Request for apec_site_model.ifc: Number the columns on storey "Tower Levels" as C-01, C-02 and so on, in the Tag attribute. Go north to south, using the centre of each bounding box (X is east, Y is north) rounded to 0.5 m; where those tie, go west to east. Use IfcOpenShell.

First a look at what the model holds.

```python
import ifcopenshell
import ifcopenshell.util.element
import ifcopenshell.util.placement

model = ifcopenshell.open("apec_site_model.ifc")
print(model.schema)
storey = next(s for s in model.by_type("IfcBuildingStorey") if s.Name == "Tower Levels")
columns = [e for e in ifcopenshell.util.element.get_decomposition(storey) if e.is_a("IfcColumn")]
for e in sorted(columns, key=lambda e: e.id()):
    origin = ifcopenshell.util.placement.get_local_placement(e.ObjectPlacement)[:3, 3]
    print(e.id(), e.Tag, e.Name, origin.round(2) + 0.0, sep=" | ")
```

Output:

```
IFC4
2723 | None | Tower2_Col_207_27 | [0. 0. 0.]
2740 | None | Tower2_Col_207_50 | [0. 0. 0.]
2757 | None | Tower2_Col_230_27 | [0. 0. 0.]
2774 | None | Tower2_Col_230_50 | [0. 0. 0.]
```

```python
import ifcopenshell
import ifcopenshell.geom
import ifcopenshell.util.element
import ifcopenshell.util.shape

model = ifcopenshell.open("apec_site_model.ifc")
settings = ifcopenshell.geom.settings()
settings.set("use-world-coords", True)


def centre(element):
    shape = ifcopenshell.geom.create_shape(settings, element)
    return ifcopenshell.util.shape.get_bbox_centroid(shape.geometry)


storey = next(s for s in model.by_type("IfcBuildingStorey") if s.Name == "Tower Levels")
columns = [e for e in ifcopenshell.util.element.get_decomposition(storey) if e.is_a("IfcColumn")]

# Insertion points can sit at a corner or the storey origin, so sort by the geometry (in metres).
centres = {e: centre(e) for e in columns}
columns.sort(key=lambda e: (-round(centres[e][1] / 0.5), centres[e][0]))

for i, e in enumerate(columns, start=1):
    number = f"C-{i:02d}"
    e.Tag = number
    print(e.id(), number)

model.write("apec_site_model_edited.ifc")
```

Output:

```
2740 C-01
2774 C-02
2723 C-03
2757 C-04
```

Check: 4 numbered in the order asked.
